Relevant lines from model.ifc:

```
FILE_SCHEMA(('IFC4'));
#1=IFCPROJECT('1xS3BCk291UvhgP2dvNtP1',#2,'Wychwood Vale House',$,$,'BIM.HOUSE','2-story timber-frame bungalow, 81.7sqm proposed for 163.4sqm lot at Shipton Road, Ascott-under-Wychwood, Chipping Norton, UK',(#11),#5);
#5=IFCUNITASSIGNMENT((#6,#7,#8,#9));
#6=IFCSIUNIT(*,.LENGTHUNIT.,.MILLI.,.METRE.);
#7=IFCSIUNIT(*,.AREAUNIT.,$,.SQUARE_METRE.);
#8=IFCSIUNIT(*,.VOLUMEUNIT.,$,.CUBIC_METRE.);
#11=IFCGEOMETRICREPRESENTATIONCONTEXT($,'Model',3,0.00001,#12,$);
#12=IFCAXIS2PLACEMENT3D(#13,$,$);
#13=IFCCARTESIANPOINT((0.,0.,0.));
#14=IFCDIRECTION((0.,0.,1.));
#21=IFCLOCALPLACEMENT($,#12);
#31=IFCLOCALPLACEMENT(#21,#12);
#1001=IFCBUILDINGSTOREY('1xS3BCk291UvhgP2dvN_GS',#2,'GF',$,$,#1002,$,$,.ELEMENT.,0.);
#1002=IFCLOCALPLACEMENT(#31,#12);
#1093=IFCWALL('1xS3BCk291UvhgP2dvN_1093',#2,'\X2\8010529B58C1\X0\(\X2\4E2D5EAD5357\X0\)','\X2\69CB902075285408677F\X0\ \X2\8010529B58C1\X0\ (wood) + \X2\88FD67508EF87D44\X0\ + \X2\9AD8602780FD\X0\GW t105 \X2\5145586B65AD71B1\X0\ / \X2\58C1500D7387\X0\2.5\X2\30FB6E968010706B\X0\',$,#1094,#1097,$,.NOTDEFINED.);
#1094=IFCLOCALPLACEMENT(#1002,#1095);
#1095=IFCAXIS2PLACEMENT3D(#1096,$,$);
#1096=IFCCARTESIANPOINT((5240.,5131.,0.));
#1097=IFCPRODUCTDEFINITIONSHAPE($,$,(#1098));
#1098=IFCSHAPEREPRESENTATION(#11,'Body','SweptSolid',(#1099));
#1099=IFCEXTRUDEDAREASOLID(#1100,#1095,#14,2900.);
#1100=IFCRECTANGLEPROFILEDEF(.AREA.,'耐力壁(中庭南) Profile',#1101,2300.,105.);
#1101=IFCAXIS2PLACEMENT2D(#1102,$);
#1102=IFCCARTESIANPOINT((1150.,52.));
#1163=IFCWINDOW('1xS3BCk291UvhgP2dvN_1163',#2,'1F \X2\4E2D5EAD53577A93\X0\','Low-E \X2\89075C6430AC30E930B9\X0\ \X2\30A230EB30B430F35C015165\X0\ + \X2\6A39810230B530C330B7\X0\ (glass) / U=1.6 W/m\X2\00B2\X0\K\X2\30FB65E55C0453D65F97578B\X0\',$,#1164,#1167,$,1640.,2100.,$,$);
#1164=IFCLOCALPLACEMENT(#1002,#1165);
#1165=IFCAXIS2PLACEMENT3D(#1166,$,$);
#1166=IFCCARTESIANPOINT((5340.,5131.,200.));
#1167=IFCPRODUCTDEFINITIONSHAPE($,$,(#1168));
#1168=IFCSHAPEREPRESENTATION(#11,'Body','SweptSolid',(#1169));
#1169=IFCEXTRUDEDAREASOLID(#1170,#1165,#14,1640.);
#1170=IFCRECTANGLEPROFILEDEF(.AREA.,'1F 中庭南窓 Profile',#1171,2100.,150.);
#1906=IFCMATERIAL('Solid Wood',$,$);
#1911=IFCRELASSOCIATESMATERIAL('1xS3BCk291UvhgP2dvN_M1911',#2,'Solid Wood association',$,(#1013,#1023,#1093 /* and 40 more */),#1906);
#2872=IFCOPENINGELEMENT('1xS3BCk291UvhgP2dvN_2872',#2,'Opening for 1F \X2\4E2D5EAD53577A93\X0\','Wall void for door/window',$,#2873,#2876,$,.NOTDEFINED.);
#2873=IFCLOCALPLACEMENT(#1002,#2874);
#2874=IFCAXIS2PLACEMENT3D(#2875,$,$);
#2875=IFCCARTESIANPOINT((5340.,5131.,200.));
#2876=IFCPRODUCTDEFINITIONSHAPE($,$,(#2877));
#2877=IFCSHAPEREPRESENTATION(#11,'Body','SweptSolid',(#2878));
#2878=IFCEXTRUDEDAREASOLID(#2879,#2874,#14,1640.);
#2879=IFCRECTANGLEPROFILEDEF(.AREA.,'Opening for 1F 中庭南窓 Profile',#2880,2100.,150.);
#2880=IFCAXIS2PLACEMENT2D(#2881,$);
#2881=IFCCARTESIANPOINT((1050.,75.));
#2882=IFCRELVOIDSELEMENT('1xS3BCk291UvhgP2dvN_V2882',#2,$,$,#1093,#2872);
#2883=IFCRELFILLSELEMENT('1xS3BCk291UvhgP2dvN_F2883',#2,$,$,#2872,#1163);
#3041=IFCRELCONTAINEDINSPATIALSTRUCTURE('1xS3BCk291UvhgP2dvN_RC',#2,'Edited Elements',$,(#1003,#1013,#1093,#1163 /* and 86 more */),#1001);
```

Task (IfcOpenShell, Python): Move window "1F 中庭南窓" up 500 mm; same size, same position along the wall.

```python
import numpy as np
import ifcopenshell
import ifcopenshell.api.geometry
import ifcopenshell.util.placement
import ifcopenshell.util.unit

model = ifcopenshell.open("model.ifc")
unit_scale = ifcopenshell.util.unit.calculate_unit_scale(model)

window = model.by_guid("1xS3BCk291UvhgP2dvN_1163")
opening = window.FillsVoids[0].RelatingOpeningElement
dz = 500.0

shift = np.array([0.0, 0.0, dz])
# The window is not placed relative to its opening, so move both.
for product in (opening, window):
    matrix = ifcopenshell.util.placement.get_local_placement(product.ObjectPlacement)
    matrix[:3, 3] += shift
    ifcopenshell.api.geometry.edit_object_placement(model, product=product, matrix=matrix, is_si=False)

print(f"moved by {dz * unit_scale:+.3f} m")

model.write("model_v2.ifc")
```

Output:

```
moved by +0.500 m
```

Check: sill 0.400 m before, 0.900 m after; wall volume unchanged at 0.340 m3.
